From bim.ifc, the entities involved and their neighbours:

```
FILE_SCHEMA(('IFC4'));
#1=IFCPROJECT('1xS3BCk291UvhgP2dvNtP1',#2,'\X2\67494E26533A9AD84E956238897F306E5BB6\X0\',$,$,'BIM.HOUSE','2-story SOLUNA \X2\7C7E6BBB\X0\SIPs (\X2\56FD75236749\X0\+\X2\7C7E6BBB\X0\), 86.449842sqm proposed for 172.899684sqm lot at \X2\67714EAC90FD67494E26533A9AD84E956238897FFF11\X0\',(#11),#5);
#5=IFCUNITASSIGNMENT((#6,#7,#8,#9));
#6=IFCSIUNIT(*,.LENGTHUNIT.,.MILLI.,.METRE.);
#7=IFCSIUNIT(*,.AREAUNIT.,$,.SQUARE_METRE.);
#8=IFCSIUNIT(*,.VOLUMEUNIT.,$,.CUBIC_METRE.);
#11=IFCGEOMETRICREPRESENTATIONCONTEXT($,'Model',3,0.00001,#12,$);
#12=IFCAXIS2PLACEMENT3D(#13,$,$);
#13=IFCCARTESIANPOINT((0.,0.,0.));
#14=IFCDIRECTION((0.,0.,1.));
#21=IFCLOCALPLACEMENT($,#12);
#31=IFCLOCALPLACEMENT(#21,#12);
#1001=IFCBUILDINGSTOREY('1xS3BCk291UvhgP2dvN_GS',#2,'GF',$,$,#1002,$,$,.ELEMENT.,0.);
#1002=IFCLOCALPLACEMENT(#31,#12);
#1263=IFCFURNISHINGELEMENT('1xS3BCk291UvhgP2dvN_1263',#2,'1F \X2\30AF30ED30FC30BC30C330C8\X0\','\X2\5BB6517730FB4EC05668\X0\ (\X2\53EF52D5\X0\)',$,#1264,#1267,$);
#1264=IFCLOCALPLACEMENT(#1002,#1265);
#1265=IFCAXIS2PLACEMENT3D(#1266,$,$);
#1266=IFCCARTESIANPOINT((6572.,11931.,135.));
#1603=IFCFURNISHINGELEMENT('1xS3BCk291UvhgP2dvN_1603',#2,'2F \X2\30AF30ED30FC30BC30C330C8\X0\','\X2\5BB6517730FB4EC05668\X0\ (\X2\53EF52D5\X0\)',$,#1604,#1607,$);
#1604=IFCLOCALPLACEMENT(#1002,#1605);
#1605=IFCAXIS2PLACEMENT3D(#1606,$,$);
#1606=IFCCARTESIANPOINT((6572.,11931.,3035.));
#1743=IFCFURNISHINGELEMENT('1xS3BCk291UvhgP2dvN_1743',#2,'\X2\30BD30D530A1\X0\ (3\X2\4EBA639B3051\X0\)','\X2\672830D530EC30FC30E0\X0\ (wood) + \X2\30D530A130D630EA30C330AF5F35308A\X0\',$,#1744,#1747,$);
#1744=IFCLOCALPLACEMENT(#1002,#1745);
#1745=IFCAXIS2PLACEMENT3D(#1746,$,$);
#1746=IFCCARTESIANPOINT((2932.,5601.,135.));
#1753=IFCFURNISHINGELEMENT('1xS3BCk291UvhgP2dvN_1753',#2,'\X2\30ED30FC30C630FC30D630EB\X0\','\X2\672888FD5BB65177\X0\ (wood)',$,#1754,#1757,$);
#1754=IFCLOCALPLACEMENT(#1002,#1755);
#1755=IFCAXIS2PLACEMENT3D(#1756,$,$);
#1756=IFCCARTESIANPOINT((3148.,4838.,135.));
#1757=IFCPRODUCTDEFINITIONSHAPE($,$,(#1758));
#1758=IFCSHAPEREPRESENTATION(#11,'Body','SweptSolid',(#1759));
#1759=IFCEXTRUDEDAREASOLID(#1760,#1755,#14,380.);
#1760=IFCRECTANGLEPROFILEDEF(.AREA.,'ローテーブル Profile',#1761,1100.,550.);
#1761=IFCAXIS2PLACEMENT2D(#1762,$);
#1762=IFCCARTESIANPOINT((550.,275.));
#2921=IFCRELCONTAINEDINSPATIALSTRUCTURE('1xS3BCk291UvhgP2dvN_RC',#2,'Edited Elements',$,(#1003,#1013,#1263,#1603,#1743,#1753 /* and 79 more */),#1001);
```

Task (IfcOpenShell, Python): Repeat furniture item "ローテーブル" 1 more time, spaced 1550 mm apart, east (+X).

```python
import numpy as np
import ifcopenshell
import ifcopenshell.api.geometry
import ifcopenshell.api.root
import ifcopenshell.util.element
import ifcopenshell.util.placement
import ifcopenshell.util.unit

model = ifcopenshell.open("bim.ifc")
unit_scale = ifcopenshell.util.unit.calculate_unit_scale(model)


def reuse_history(source, copy):
    """copy_class also copies each property set's owner history, people and application; keep the originals."""
    for rel in copy.IsDefinedBy:
        if rel.is_a("IfcRelDefinesByProperties") and (history := rel.RelatingPropertyDefinition.OwnerHistory):
            rel.RelatingPropertyDefinition.OwnerHistory = source.OwnerHistory
            ifcopenshell.util.element.remove_deep2(model, history)


source = model.by_id(1753)
base = ifcopenshell.util.placement.get_local_placement(source.ObjectPlacement)
step = np.array([1.0, 0.0, 0.0]) * 1.55 / unit_scale

for i in range(1, 2):
    copy = ifcopenshell.api.root.copy_class(model, product=source)
    copy.Representation = ifcopenshell.util.element.copy_deep(
        model, source.Representation, exclude=["IfcGeometricRepresentationContext", "IfcRepresentationMap"]
    )
    reuse_history(source, copy)
    matrix = base.copy()
    matrix[:3, 3] += i * step
    print("added at", matrix[:3, 3].round(3) + 0.0)
    ifcopenshell.api.geometry.edit_object_placement(model, product=copy, matrix=matrix, is_si=False)

model.write("bim-out.ifc")
```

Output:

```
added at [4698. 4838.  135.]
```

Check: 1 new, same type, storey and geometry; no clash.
